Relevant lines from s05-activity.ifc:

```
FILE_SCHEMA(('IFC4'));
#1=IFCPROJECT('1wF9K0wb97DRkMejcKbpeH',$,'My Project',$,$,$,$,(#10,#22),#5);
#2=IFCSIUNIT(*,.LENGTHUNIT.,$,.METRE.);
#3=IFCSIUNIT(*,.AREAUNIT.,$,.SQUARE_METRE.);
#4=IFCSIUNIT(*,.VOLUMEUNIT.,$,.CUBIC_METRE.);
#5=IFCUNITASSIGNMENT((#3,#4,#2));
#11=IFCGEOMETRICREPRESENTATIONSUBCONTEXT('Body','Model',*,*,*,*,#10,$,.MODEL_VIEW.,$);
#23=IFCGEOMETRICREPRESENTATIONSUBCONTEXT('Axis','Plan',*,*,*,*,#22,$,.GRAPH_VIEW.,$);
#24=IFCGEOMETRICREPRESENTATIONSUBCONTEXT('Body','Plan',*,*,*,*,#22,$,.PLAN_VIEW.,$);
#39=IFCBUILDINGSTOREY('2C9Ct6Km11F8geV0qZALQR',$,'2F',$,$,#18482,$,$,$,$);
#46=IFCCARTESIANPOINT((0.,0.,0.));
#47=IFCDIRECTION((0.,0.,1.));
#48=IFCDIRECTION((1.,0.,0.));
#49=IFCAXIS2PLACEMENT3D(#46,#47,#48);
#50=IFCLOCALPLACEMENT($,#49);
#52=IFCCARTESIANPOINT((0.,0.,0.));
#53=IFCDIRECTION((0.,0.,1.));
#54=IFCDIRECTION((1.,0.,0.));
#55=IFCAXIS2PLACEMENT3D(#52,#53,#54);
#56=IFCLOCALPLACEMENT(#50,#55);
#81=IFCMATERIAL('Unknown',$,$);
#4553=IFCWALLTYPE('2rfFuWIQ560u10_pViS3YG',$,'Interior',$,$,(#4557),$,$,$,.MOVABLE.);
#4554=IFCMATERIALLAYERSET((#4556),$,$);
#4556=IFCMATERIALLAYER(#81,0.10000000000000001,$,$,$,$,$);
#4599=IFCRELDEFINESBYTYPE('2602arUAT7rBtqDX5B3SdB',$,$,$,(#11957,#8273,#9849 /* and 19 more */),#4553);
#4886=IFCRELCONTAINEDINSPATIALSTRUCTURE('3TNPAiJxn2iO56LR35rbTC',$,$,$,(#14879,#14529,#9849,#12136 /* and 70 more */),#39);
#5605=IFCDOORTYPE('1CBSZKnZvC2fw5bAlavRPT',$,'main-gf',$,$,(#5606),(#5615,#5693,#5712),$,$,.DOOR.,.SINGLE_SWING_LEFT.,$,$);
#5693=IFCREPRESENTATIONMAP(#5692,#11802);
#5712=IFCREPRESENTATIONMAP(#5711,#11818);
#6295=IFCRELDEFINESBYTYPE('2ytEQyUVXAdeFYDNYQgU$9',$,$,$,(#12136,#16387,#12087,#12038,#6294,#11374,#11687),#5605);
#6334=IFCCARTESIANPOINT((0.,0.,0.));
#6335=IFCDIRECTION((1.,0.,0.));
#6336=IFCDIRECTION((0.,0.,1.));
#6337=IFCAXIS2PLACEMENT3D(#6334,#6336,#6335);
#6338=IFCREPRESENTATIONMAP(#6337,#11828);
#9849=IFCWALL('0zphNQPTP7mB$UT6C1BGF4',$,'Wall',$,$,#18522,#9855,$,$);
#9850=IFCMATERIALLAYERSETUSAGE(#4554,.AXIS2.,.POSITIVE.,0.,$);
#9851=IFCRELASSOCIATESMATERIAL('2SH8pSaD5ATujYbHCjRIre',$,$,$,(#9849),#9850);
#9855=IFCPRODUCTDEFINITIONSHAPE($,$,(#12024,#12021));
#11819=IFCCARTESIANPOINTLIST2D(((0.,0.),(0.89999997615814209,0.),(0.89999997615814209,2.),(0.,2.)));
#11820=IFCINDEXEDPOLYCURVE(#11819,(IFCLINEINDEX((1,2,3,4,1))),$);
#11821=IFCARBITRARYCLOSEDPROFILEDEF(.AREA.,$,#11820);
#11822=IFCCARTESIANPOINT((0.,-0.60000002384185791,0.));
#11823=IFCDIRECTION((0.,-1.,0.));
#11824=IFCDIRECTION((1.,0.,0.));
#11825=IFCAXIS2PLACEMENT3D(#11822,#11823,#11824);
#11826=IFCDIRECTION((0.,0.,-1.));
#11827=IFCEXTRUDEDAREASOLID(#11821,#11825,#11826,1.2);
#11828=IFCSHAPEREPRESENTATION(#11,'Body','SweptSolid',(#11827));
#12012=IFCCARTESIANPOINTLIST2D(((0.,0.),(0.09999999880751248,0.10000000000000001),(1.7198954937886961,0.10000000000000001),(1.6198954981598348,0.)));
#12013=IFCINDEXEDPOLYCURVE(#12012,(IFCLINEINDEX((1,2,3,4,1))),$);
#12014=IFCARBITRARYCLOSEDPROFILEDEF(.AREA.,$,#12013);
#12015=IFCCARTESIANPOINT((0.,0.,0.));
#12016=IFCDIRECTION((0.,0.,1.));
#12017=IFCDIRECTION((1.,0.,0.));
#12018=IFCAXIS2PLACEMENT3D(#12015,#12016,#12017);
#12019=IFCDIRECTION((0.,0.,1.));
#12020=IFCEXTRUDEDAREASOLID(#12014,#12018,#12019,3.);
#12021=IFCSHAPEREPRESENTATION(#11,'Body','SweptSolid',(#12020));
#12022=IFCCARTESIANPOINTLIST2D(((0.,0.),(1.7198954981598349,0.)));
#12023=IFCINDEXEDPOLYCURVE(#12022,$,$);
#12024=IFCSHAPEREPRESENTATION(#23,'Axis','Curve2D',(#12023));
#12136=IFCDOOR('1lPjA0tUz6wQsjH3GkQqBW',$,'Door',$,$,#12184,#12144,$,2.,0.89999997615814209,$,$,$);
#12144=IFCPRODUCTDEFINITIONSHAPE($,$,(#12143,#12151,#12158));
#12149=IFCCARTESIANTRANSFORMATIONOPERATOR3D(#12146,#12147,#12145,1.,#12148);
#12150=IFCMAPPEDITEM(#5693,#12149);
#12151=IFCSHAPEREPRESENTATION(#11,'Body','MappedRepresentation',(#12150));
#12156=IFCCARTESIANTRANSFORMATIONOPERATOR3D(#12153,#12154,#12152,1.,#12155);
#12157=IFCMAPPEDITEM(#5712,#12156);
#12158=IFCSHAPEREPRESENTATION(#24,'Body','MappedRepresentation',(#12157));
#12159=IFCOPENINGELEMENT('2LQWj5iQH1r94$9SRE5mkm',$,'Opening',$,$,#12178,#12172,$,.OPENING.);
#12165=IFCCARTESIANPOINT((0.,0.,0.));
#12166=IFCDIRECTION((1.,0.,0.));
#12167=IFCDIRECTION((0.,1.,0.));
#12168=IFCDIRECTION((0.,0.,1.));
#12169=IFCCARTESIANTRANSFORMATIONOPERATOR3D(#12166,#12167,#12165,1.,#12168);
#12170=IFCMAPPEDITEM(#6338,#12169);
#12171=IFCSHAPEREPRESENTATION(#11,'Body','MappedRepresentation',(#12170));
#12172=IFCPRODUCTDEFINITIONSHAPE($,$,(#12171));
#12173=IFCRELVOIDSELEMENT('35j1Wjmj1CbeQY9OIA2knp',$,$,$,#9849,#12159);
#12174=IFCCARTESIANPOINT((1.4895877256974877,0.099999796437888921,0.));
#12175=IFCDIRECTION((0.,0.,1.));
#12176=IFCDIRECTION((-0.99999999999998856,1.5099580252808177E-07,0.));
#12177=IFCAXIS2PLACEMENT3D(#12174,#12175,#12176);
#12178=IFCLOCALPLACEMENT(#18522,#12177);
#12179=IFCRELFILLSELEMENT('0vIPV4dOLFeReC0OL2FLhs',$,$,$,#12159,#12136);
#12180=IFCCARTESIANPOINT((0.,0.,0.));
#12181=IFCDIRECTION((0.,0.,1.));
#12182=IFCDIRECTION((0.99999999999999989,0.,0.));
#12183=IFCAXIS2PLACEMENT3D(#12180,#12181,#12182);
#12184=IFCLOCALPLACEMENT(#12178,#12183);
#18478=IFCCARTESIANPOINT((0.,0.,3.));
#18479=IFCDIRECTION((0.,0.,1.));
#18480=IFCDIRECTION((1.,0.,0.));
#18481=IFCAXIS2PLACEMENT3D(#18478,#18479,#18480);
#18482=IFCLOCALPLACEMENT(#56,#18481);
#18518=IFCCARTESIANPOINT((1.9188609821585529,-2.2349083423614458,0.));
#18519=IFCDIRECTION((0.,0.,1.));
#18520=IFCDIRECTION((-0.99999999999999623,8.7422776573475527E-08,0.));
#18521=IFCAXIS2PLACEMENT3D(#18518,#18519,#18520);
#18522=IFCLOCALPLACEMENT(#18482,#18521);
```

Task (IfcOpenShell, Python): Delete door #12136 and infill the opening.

```python
import ifcopenshell
import ifcopenshell.api.feature
import ifcopenshell.api.root
import ifcopenshell.geom
import ifcopenshell.util.shape

model = ifcopenshell.open("s05-activity.ifc")
settings = ifcopenshell.geom.settings()


def volume(element):
    """Net volume in cubic metres, openings subtracted."""
    shape = ifcopenshell.geom.create_shape(settings, element)
    return ifcopenshell.util.shape.get_volume(shape.geometry)


door = model.by_guid("1lPjA0tUz6wQsjH3GkQqBW")
opening = door.FillsVoids[0].RelatingOpeningElement
wall = opening.VoidsElements[0].RelatingBuildingElement
before = volume(wall)

ifcopenshell.api.root.remove_product(model, product=door)
ifcopenshell.api.feature.remove_feature(model, feature=opening)

after = volume(wall)

print(f"wall volume {before:.3f} -> {after:.3f} m3")

model.write("s05-activity-out.ifc")
```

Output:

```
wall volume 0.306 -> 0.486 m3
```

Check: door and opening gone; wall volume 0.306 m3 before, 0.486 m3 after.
